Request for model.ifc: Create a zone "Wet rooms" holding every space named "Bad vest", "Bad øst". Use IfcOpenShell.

First a look at what the model holds.

```python
import ifcopenshell

model = ifcopenshell.open("model.ifc")
print(model.schema)
seen = {}
for space in model.by_type("IfcSpace"):
    seen[space.LongName] = seen.get(space.LongName, 0) + 1
for name, count in sorted(seen.items(), key=str):
    print(count, "x", name)
print("zones:", [z.Name for z in model.by_type("IfcZone")][:20])
```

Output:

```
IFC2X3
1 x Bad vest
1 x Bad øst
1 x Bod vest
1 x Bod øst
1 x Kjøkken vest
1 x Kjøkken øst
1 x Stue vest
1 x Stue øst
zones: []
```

```python
import ifcopenshell
import ifcopenshell.api.group
import ifcopenshell.api.root

model = ifcopenshell.open("model.ifc")

names = {"Bad vest", "Bad øst"}
spaces = [s for s in model.by_type("IfcSpace") if s.LongName in names]

zone = ifcopenshell.api.root.create_entity(model, ifc_class="IfcZone", name="Wet rooms")
ifcopenshell.api.group.assign_group(model, products=spaces, group=zone)
print(len(spaces), "spaces in", zone.Name)

model.write("model_edited.ifc")
```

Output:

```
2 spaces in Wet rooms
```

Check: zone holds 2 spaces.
